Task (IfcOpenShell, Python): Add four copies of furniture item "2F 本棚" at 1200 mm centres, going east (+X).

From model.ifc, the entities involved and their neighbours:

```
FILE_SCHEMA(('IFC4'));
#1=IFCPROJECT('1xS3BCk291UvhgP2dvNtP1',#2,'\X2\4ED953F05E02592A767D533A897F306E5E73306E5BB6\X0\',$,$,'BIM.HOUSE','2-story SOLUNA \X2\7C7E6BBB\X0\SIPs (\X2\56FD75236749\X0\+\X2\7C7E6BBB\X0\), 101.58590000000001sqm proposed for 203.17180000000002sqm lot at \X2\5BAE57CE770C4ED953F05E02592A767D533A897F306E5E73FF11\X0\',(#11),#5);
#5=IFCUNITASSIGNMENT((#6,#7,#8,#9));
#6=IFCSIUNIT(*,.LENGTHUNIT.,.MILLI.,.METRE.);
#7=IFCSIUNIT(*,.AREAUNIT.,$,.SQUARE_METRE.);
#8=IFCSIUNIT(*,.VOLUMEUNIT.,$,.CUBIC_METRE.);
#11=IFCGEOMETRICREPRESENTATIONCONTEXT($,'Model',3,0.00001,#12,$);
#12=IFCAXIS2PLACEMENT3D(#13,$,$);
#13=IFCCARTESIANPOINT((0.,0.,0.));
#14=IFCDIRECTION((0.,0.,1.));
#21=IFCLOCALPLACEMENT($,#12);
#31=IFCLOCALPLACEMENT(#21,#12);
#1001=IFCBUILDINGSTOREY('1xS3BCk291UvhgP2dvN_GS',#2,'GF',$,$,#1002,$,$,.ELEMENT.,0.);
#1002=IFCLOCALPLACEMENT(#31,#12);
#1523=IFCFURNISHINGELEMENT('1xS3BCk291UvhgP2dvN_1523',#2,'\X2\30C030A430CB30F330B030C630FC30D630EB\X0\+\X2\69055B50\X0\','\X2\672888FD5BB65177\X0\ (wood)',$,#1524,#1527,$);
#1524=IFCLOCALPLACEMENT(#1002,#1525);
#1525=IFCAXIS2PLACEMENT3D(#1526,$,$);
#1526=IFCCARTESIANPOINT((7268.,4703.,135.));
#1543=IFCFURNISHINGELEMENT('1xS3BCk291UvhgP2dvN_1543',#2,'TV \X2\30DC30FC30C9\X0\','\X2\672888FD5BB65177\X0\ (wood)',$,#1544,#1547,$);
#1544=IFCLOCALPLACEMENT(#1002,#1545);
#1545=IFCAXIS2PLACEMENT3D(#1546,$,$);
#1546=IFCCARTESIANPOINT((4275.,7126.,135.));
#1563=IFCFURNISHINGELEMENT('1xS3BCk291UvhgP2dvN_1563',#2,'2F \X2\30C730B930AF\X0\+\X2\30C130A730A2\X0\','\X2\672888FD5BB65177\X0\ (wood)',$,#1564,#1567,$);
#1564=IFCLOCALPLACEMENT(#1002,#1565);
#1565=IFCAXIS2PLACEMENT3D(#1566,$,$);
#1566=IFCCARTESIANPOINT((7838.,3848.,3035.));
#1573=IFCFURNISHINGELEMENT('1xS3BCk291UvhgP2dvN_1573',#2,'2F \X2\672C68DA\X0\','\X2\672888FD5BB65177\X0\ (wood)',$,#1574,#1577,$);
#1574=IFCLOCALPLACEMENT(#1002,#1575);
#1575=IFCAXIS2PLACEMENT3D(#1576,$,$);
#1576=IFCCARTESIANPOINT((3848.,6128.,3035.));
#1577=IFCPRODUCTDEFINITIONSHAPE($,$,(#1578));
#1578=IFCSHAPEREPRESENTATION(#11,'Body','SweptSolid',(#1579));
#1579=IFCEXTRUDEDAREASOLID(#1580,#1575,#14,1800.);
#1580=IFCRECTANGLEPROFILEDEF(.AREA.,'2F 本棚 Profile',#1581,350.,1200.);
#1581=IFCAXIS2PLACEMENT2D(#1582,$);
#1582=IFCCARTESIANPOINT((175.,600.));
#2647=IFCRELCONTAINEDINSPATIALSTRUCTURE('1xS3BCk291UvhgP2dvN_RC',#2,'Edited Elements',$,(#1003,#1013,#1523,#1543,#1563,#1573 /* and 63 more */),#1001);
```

```python
import numpy as np
import ifcopenshell
import ifcopenshell.api.geometry
import ifcopenshell.api.root
import ifcopenshell.util.element
import ifcopenshell.util.placement

model = ifcopenshell.open("model.ifc")


def reuse_history(source, copy):
    """copy_class also copies each property set's owner history, people and application; keep the originals."""
    for rel in copy.IsDefinedBy:
        if rel.is_a("IfcRelDefinesByProperties") and (history := rel.RelatingPropertyDefinition.OwnerHistory):
            rel.RelatingPropertyDefinition.OwnerHistory = source.OwnerHistory
            ifcopenshell.util.element.remove_deep2(model, history)


source = model.by_guid("1xS3BCk291UvhgP2dvN_1573")
base = ifcopenshell.util.placement.get_local_placement(source.ObjectPlacement)
step = np.array([1.0, 0.0, 0.0]) * 1200.0

for i in range(1, 5):
    copy = ifcopenshell.api.root.copy_class(model, product=source)
    copy.Representation = ifcopenshell.util.element.copy_deep(
        model, source.Representation, exclude=["IfcGeometricRepresentationContext", "IfcRepresentationMap"]
    )
    reuse_history(source, copy)
    matrix = base.copy()
    matrix[:3, 3] += i * step
    print("added at", matrix[:3, 3].round(3) + 0.0)
    ifcopenshell.api.geometry.edit_object_placement(model, product=copy, matrix=matrix, is_si=False)

model.write("model-out.ifc")
```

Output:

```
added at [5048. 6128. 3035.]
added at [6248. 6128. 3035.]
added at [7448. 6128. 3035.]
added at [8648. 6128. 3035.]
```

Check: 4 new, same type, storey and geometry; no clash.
